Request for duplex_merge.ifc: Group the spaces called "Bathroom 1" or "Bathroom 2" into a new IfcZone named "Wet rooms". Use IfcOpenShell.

First a look at what the model holds.

```python
import ifcopenshell

model = ifcopenshell.open("duplex_merge.ifc")
print(model.schema)
seen = {}
for space in model.by_type("IfcSpace"):
    seen[space.LongName] = seen.get(space.LongName, 0) + 1
for name, count in sorted(seen.items(), key=str):
    print(count, "x", name)
print("zones:", [z.Name for z in model.by_type("IfcZone")][:20])
```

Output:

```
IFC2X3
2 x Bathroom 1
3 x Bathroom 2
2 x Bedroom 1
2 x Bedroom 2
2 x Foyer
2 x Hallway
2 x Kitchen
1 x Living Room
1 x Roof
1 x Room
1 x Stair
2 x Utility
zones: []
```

```python
import ifcopenshell
import ifcopenshell.api.group
import ifcopenshell.api.root

model = ifcopenshell.open("duplex_merge.ifc")

names = {"Bathroom 1", "Bathroom 2"}
spaces = [s for s in model.by_type("IfcSpace") if s.LongName in names]

zone = ifcopenshell.api.root.create_entity(model, ifc_class="IfcZone", name="Wet rooms")
ifcopenshell.api.group.assign_group(model, products=spaces, group=zone)
print(len(spaces), "spaces in", zone.Name)

model.write("duplex_merge-out.ifc")
```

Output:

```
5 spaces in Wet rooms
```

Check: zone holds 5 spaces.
